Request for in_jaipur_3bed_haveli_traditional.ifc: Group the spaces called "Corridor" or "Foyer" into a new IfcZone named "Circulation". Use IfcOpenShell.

First a look at what the model holds.

```python
import ifcopenshell

model = ifcopenshell.open("in_jaipur_3bed_haveli_traditional.ifc")
print(model.schema)
seen = {}
for space in model.by_type("IfcSpace"):
    seen[space.LongName] = seen.get(space.LongName, 0) + 1
for name, count in sorted(seen.items(), key=str):
    print(count, "x", name)
print("zones:", [z.Name for z in model.by_type("IfcZone")][:20])
```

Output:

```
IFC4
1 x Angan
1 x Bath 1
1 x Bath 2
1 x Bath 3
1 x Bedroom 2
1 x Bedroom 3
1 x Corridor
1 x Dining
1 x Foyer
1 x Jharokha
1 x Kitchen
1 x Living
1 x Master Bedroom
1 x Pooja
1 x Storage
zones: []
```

```python
import ifcopenshell
import ifcopenshell.api.group
import ifcopenshell.api.root

model = ifcopenshell.open("in_jaipur_3bed_haveli_traditional.ifc")

names = {"Corridor", "Foyer"}
spaces = [s for s in model.by_type("IfcSpace") if s.LongName in names]

zone = ifcopenshell.api.root.create_entity(model, ifc_class="IfcZone", name="Circulation")
ifcopenshell.api.group.assign_group(model, products=spaces, group=zone)
print(len(spaces), "spaces in", zone.Name)

model.write("in_jaipur_3bed_haveli_traditional_updated.ifc")
```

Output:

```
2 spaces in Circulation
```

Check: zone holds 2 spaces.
